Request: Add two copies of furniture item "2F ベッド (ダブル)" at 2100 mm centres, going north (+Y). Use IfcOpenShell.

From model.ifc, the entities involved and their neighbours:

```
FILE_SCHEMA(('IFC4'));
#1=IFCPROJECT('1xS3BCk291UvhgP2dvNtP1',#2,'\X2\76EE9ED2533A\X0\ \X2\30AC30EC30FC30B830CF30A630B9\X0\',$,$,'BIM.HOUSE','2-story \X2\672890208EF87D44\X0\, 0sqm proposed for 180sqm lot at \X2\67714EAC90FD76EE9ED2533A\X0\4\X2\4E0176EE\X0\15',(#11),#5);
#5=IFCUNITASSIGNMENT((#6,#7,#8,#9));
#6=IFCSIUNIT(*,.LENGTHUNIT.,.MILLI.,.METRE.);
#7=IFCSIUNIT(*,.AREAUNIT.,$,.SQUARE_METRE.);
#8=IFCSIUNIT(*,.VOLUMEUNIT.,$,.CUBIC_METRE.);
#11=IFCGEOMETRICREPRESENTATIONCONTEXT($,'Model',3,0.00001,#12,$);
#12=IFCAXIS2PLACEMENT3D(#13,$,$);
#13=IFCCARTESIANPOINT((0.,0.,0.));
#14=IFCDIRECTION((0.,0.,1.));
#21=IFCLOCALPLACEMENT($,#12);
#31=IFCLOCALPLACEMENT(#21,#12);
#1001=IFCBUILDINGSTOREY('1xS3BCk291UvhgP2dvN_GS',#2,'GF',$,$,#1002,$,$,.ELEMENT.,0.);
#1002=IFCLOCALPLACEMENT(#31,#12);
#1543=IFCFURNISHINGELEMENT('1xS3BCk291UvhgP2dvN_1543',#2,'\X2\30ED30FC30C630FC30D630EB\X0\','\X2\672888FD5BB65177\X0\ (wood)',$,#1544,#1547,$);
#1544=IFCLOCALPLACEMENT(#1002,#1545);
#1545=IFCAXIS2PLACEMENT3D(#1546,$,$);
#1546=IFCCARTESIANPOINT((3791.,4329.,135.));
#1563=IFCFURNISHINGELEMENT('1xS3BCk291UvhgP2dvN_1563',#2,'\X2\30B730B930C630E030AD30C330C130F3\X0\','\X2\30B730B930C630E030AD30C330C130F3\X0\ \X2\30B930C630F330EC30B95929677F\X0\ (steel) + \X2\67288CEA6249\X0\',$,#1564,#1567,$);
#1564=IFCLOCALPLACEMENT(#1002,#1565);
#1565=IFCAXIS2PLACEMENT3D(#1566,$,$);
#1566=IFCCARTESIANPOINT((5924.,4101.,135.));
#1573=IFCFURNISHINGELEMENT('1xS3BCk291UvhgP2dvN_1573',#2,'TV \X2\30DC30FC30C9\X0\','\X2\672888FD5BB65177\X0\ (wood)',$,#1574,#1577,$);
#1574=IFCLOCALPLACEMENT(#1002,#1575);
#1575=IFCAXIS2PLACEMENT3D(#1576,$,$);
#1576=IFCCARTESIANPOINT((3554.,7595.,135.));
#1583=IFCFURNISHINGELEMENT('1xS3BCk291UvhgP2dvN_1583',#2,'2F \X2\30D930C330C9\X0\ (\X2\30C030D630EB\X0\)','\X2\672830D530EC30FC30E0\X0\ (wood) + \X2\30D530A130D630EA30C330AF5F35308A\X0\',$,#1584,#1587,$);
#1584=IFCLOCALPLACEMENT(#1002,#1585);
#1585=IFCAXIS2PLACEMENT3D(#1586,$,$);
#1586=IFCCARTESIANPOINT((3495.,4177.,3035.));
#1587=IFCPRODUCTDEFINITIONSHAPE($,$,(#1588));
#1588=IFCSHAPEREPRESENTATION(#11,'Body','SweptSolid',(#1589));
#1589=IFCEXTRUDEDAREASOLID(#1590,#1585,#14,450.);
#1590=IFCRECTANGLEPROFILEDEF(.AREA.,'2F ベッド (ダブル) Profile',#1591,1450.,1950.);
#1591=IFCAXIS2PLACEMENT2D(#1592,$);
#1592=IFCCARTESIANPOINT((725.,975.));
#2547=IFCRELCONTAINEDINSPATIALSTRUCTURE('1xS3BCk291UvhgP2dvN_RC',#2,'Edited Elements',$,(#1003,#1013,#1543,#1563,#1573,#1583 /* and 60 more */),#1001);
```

```python
import numpy as np
import ifcopenshell
import ifcopenshell.api.geometry
import ifcopenshell.api.root
import ifcopenshell.util.element
import ifcopenshell.util.placement
import ifcopenshell.util.unit

model = ifcopenshell.open("model.ifc")
unit_scale = ifcopenshell.util.unit.calculate_unit_scale(model)


def reuse_history(source, copy):
    """copy_class also copies each property set's owner history, people and application; keep the originals."""
    for rel in copy.IsDefinedBy:
        if rel.is_a("IfcRelDefinesByProperties") and (history := rel.RelatingPropertyDefinition.OwnerHistory):
            rel.RelatingPropertyDefinition.OwnerHistory = source.OwnerHistory
            ifcopenshell.util.element.remove_deep2(model, history)


source = model.by_id(1583)
base = ifcopenshell.util.placement.get_local_placement(source.ObjectPlacement)
step = np.array([0.0, 1.0, 0.0]) * 2.1 / unit_scale

for i in range(1, 3):
    copy = ifcopenshell.api.root.copy_class(model, product=source)
    copy.Representation = ifcopenshell.util.element.copy_deep(
        model, source.Representation, exclude=["IfcGeometricRepresentationContext", "IfcRepresentationMap"]
    )
    reuse_history(source, copy)
    matrix = base.copy()
    matrix[:3, 3] += i * step
    print("added at", matrix[:3, 3].round(3) + 0.0)
    ifcopenshell.api.geometry.edit_object_placement(model, product=copy, matrix=matrix, is_si=False)

model.write("model_updated.ifc")
```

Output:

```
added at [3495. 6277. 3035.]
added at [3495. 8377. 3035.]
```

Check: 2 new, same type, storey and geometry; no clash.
